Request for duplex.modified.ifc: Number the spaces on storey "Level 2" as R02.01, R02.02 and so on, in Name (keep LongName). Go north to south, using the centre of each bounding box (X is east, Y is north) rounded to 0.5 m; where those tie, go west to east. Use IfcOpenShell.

First a look at what the model holds.

```python
import ifcopenshell
import ifcopenshell.util.element
import ifcopenshell.util.placement

model = ifcopenshell.open("duplex.modified.ifc")
print(model.schema)
storey = next(s for s in model.by_type("IfcBuildingStorey") if s.Name == "Level 2")
spaces = [e for e in ifcopenshell.util.element.get_decomposition(storey) if e.is_a("IfcSpace")]
for e in sorted(spaces, key=lambda e: e.id()):
    origin = ifcopenshell.util.placement.get_local_placement(e.ObjectPlacement)[:3, 3]
    print(e.id(), e.Name, e.LongName, origin.round(2) + 0.0, sep=" | ")
```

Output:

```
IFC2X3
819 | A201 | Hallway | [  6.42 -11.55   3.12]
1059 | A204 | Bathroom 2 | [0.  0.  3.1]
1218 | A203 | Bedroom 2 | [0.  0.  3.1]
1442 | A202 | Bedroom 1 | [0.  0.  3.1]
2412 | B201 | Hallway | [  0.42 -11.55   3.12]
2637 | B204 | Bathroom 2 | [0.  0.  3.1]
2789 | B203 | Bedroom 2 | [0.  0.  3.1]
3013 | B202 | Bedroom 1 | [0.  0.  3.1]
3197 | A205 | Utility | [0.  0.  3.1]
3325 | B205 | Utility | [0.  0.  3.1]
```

```python
import ifcopenshell
import ifcopenshell.geom
import ifcopenshell.util.element
import ifcopenshell.util.shape

model = ifcopenshell.open("duplex.modified.ifc")
settings = ifcopenshell.geom.settings()
settings.set("use-world-coords", True)


def centre(element):
    shape = ifcopenshell.geom.create_shape(settings, element)
    return ifcopenshell.util.shape.get_bbox_centroid(shape.geometry)


storey = next(s for s in model.by_type("IfcBuildingStorey") if s.Name == "Level 2")
spaces = [e for e in ifcopenshell.util.element.get_decomposition(storey) if e.is_a("IfcSpace")]

# Insertion points can sit at a corner or the storey origin, so sort by the geometry (in metres).
centres = {e: centre(e) for e in spaces}
spaces.sort(key=lambda e: (-round(centres[e][1] / 0.5), centres[e][0]))

for i, e in enumerate(spaces, start=1):
    number = f"R02.{i:02d}"
    e.Name = number
    print(e.id(), number)

model.write("duplex.modified_v2.ifc")
```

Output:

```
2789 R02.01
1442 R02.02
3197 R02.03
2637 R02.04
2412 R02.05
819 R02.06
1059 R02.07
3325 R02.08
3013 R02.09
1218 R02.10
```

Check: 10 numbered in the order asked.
